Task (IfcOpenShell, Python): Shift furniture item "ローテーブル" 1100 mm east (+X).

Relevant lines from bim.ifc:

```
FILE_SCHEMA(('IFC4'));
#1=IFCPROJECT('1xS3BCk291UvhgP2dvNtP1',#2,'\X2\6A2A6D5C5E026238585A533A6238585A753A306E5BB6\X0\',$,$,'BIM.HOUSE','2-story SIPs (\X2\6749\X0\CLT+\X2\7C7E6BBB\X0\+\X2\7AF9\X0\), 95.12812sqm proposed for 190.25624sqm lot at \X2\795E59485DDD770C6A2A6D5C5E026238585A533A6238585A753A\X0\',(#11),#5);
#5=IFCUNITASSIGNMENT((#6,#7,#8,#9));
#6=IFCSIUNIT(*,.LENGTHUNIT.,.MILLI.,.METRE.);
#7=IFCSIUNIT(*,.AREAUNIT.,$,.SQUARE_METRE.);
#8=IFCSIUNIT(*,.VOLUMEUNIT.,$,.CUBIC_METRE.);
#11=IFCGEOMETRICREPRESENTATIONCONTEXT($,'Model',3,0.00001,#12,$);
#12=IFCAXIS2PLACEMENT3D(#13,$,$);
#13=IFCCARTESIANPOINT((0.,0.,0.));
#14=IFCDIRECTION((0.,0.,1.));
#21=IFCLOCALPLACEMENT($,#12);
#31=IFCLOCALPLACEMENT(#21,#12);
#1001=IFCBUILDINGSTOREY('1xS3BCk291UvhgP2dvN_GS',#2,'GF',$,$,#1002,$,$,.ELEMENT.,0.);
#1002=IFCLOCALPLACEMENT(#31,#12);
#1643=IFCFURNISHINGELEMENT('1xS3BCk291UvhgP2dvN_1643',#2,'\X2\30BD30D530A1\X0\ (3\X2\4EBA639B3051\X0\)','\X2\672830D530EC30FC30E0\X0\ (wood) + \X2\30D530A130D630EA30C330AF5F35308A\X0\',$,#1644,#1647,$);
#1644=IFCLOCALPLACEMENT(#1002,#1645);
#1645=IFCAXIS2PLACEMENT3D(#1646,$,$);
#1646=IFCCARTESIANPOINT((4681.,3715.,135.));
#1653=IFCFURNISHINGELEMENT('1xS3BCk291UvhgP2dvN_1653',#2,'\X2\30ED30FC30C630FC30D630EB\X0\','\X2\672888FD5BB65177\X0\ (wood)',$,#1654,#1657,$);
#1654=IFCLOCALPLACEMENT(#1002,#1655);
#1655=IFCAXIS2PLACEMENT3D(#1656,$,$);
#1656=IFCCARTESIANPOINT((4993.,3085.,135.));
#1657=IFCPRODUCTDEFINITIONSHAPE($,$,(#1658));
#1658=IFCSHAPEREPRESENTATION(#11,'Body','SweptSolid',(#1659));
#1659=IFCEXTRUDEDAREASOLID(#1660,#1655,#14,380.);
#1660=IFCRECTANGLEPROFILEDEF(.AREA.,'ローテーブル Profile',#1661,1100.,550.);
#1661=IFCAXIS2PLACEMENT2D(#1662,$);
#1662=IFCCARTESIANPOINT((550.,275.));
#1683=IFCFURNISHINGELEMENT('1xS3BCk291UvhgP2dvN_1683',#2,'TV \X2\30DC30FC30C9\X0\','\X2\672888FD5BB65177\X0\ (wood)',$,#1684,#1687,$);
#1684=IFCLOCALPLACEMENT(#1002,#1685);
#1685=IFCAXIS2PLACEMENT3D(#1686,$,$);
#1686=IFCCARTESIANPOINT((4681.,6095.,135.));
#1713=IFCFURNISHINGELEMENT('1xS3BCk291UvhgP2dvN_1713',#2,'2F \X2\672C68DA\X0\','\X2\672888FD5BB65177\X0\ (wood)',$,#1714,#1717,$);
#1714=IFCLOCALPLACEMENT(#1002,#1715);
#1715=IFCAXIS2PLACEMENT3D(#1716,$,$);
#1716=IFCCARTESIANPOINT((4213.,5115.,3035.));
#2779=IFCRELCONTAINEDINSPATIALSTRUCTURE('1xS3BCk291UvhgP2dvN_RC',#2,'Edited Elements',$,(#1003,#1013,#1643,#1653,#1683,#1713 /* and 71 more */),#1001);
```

```python
import ifcopenshell
import ifcopenshell.api.geometry
import ifcopenshell.util.placement
import ifcopenshell.util.unit

model = ifcopenshell.open("bim.ifc")
unit_scale = ifcopenshell.util.unit.calculate_unit_scale(model)

item = model.by_guid("1xS3BCk291UvhgP2dvN_1653")
matrix = ifcopenshell.util.placement.get_local_placement(item.ObjectPlacement)
matrix[0, 3] += 1.1 / unit_scale
ifcopenshell.api.geometry.edit_object_placement(model, product=item, matrix=matrix, is_si=False)

print(ifcopenshell.util.placement.get_local_placement(item.ObjectPlacement).round(3) + 0.0)

model.write("bim_rev.ifc")
```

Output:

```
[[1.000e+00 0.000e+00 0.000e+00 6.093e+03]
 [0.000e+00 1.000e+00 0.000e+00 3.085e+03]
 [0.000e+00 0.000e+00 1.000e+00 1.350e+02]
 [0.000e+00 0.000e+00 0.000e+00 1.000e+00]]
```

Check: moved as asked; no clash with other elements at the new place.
